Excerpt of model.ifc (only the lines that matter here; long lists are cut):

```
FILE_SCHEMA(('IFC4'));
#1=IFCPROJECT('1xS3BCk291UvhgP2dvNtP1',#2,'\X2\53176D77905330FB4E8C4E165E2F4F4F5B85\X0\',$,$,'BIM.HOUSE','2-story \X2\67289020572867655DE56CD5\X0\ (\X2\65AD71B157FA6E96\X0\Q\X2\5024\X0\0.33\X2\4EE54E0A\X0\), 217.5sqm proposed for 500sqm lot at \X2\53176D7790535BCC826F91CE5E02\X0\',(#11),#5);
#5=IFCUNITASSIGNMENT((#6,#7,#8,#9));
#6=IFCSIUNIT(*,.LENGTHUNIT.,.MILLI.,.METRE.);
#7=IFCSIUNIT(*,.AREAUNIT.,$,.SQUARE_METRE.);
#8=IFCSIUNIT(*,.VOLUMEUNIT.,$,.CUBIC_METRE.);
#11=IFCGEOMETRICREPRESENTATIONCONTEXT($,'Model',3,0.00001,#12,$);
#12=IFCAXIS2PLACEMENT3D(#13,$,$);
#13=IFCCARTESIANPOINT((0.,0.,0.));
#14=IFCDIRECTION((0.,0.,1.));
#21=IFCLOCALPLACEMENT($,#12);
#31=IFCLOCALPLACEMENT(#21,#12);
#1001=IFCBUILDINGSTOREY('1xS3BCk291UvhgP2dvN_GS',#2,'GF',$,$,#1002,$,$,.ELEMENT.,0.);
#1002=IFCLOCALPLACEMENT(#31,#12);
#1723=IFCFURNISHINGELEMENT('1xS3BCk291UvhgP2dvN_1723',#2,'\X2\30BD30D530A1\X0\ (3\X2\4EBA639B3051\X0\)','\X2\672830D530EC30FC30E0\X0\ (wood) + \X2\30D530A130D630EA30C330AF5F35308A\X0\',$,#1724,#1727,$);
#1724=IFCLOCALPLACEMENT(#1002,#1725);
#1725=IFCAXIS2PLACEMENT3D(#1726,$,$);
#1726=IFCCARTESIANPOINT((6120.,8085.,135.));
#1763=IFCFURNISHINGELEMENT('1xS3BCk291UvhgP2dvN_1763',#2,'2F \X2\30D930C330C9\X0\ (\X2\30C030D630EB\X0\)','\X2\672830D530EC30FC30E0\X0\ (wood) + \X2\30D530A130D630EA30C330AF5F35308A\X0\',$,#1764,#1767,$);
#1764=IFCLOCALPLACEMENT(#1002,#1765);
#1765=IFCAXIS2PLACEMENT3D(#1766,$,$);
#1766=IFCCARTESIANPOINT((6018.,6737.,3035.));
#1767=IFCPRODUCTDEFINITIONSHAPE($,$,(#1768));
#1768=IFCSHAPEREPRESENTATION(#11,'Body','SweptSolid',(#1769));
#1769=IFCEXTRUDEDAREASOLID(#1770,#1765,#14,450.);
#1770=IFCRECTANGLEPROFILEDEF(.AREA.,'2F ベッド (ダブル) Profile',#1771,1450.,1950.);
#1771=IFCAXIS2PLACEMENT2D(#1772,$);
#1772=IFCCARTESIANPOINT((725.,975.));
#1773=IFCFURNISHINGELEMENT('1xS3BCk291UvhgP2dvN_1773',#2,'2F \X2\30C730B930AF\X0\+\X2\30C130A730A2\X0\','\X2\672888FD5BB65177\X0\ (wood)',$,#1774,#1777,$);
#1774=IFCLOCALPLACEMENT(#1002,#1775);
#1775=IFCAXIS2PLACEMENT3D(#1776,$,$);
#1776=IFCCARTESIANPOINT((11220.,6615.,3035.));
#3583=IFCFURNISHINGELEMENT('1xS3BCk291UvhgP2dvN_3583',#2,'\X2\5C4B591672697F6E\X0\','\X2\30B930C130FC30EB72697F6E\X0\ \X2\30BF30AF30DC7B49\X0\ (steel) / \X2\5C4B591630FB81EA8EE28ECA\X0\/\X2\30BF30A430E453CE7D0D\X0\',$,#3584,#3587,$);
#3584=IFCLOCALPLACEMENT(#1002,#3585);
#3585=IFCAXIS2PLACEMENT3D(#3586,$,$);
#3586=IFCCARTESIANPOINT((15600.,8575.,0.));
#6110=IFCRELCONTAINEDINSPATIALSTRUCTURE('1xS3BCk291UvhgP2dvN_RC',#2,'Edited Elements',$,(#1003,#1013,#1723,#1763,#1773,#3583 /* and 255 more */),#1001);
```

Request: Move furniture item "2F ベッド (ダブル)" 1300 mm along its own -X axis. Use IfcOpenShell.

```python
import ifcopenshell
import ifcopenshell.api.geometry
import ifcopenshell.util.placement
import ifcopenshell.util.unit

model = ifcopenshell.open("model.ifc")
unit_scale = ifcopenshell.util.unit.calculate_unit_scale(model)

item = model.by_guid("1xS3BCk291UvhgP2dvN_1763")
matrix = ifcopenshell.util.placement.get_local_placement(item.ObjectPlacement)
matrix[:3, 3] -= matrix[:3, 0] * 1.3 / unit_scale
ifcopenshell.api.geometry.edit_object_placement(model, product=item, matrix=matrix, is_si=False)

print(ifcopenshell.util.placement.get_local_placement(item.ObjectPlacement).round(3) + 0.0)

model.write("model_v2.ifc")
```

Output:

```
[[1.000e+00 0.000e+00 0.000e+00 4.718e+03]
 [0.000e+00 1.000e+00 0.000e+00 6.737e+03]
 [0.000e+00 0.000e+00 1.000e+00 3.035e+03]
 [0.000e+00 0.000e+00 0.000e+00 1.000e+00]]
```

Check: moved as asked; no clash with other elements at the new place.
